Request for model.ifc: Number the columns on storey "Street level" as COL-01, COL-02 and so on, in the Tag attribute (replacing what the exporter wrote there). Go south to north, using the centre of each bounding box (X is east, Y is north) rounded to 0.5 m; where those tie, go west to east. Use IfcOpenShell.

First a look at what the model holds.

```python
import ifcopenshell
import ifcopenshell.util.element
import ifcopenshell.util.placement

model = ifcopenshell.open("model.ifc")
print(model.schema)
storey = next(s for s in model.by_type("IfcBuildingStorey") if s.Name == "Street level")
columns = [e for e in ifcopenshell.util.element.get_decomposition(storey) if e.is_a("IfcColumn")]
for e in sorted(columns, key=lambda e: e.id()):
    origin = ifcopenshell.util.placement.get_local_placement(e.ObjectPlacement)[:3, 3]
    print(e.id(), e.Tag, e.Name, origin.round(2) + 0.0, sep=" | ")
```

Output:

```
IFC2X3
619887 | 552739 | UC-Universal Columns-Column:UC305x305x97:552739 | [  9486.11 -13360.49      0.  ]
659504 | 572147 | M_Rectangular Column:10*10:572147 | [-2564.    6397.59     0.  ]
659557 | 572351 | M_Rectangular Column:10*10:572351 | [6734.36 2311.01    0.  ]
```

```python
import ifcopenshell
import ifcopenshell.geom
import ifcopenshell.util.element
import ifcopenshell.util.shape

model = ifcopenshell.open("model.ifc")
settings = ifcopenshell.geom.settings()
settings.set("use-world-coords", True)


def centre(element):
    shape = ifcopenshell.geom.create_shape(settings, element)
    return ifcopenshell.util.shape.get_bbox_centroid(shape.geometry)


storey = next(s for s in model.by_type("IfcBuildingStorey") if s.Name == "Street level")
columns = [e for e in ifcopenshell.util.element.get_decomposition(storey) if e.is_a("IfcColumn")]

# Insertion points can sit at a corner or the storey origin, so sort by the geometry (in metres).
centres = {e: centre(e) for e in columns}
columns.sort(key=lambda e: (round(centres[e][1] / 0.5), centres[e][0]))

for i, e in enumerate(columns, start=1):
    number = f"COL-{i:02d}"
    e.Tag = number
    print(e.id(), number)

model.write("model_rev.ifc")
```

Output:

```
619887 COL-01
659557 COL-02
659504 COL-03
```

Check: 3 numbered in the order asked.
